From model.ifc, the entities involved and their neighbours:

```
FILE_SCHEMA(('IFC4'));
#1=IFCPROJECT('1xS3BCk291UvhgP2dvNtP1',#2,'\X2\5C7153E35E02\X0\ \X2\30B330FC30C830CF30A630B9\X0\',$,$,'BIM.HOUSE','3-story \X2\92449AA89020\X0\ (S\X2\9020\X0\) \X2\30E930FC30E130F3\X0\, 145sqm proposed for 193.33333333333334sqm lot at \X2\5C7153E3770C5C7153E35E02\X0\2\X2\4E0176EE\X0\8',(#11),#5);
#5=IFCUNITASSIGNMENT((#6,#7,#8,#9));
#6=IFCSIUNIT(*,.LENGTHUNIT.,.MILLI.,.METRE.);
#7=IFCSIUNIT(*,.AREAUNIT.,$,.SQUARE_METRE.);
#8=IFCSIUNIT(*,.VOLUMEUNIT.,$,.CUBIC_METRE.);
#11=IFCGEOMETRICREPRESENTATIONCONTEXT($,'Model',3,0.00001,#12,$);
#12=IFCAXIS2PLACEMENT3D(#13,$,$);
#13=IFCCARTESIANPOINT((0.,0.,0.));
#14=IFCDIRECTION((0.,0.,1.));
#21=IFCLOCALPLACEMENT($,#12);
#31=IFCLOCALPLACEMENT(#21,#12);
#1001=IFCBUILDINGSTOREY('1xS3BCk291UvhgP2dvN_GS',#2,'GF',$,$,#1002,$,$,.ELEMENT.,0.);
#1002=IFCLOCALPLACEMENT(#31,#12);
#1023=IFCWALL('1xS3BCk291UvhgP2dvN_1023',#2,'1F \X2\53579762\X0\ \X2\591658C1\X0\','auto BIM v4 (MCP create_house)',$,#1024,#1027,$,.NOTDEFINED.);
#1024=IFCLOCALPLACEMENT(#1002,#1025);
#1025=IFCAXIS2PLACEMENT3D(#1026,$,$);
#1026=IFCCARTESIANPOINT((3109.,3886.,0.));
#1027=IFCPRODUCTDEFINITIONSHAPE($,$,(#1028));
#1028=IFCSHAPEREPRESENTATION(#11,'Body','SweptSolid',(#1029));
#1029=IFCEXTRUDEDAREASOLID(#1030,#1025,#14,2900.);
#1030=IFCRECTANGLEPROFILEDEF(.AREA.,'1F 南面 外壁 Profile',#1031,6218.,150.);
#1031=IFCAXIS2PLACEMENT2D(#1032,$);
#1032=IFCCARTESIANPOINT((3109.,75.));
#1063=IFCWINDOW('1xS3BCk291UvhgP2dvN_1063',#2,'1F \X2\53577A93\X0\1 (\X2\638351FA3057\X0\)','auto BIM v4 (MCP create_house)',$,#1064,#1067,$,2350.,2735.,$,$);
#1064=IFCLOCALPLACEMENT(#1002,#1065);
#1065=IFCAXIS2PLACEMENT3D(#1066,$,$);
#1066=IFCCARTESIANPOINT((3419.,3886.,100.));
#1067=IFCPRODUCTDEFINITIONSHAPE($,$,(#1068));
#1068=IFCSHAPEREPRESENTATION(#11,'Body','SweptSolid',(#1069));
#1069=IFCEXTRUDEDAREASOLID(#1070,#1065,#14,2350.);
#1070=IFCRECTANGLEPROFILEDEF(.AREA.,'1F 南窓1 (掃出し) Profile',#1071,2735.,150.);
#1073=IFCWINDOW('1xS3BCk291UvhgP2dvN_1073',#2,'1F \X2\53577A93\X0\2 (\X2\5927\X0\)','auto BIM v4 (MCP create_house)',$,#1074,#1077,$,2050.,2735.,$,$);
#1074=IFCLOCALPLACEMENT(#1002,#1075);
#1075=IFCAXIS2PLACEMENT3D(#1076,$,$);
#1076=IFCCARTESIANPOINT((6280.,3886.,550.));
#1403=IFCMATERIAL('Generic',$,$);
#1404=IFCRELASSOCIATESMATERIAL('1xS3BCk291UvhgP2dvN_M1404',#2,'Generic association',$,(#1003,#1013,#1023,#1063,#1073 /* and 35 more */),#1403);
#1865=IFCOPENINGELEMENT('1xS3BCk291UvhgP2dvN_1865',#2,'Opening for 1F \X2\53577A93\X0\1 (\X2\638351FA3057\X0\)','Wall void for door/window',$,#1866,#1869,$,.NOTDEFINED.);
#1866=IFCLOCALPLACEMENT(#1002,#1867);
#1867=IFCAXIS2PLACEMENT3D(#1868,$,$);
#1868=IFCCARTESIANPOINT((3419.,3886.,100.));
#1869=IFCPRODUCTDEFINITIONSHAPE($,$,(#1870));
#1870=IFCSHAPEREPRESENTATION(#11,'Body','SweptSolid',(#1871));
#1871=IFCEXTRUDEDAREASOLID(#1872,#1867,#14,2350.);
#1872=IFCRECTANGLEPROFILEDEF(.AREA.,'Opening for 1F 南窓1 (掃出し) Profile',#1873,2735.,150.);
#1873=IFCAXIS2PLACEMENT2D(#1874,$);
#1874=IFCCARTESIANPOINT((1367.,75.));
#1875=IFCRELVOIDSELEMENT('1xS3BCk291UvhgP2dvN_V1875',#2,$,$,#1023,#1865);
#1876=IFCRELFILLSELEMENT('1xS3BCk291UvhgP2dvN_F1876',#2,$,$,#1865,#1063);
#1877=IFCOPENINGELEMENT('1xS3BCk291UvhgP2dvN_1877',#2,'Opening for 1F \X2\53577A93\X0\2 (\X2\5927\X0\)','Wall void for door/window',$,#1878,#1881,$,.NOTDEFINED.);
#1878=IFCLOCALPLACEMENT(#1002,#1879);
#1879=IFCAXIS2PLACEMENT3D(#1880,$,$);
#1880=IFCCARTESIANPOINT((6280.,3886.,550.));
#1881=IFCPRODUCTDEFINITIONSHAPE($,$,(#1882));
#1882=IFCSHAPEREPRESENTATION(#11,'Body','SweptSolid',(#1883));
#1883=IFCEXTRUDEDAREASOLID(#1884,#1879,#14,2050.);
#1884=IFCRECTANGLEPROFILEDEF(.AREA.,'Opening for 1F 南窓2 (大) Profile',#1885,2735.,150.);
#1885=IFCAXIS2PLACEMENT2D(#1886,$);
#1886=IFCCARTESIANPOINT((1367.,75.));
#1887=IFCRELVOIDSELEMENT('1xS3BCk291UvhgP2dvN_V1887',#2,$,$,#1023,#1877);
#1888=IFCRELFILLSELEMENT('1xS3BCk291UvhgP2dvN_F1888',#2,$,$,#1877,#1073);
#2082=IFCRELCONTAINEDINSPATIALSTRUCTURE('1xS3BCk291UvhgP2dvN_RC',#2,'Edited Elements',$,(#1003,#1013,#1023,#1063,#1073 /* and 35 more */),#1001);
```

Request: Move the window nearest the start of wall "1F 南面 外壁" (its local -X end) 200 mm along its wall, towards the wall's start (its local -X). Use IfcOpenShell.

```python
import ifcopenshell
import ifcopenshell.api.geometry
import ifcopenshell.util.placement

model = ifcopenshell.open("model.ifc")

window = model.by_id(1063)
opening = window.FillsVoids[0].RelatingOpeningElement
wall = opening.VoidsElements[0].RelatingBuildingElement

wall_matrix = ifcopenshell.util.placement.get_local_placement(wall.ObjectPlacement)
shift = wall_matrix[:3, 0] * -200.0
before = ifcopenshell.util.placement.get_local_placement(window.ObjectPlacement)[:3, 3].copy()

# The window is not placed relative to its opening, so move both.
for product in (opening, window):
    matrix = ifcopenshell.util.placement.get_local_placement(product.ObjectPlacement)
    matrix[:3, 3] += shift
    ifcopenshell.api.geometry.edit_object_placement(model, product=product, matrix=matrix, is_si=False)

after = ifcopenshell.util.placement.get_local_placement(window.ObjectPlacement)[:3, 3]
print("window moved by", (after - before).round(3) + 0.0)

model.write("model_rev.ifc")
```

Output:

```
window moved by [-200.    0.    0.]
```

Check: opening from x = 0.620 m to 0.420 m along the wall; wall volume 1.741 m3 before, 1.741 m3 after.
